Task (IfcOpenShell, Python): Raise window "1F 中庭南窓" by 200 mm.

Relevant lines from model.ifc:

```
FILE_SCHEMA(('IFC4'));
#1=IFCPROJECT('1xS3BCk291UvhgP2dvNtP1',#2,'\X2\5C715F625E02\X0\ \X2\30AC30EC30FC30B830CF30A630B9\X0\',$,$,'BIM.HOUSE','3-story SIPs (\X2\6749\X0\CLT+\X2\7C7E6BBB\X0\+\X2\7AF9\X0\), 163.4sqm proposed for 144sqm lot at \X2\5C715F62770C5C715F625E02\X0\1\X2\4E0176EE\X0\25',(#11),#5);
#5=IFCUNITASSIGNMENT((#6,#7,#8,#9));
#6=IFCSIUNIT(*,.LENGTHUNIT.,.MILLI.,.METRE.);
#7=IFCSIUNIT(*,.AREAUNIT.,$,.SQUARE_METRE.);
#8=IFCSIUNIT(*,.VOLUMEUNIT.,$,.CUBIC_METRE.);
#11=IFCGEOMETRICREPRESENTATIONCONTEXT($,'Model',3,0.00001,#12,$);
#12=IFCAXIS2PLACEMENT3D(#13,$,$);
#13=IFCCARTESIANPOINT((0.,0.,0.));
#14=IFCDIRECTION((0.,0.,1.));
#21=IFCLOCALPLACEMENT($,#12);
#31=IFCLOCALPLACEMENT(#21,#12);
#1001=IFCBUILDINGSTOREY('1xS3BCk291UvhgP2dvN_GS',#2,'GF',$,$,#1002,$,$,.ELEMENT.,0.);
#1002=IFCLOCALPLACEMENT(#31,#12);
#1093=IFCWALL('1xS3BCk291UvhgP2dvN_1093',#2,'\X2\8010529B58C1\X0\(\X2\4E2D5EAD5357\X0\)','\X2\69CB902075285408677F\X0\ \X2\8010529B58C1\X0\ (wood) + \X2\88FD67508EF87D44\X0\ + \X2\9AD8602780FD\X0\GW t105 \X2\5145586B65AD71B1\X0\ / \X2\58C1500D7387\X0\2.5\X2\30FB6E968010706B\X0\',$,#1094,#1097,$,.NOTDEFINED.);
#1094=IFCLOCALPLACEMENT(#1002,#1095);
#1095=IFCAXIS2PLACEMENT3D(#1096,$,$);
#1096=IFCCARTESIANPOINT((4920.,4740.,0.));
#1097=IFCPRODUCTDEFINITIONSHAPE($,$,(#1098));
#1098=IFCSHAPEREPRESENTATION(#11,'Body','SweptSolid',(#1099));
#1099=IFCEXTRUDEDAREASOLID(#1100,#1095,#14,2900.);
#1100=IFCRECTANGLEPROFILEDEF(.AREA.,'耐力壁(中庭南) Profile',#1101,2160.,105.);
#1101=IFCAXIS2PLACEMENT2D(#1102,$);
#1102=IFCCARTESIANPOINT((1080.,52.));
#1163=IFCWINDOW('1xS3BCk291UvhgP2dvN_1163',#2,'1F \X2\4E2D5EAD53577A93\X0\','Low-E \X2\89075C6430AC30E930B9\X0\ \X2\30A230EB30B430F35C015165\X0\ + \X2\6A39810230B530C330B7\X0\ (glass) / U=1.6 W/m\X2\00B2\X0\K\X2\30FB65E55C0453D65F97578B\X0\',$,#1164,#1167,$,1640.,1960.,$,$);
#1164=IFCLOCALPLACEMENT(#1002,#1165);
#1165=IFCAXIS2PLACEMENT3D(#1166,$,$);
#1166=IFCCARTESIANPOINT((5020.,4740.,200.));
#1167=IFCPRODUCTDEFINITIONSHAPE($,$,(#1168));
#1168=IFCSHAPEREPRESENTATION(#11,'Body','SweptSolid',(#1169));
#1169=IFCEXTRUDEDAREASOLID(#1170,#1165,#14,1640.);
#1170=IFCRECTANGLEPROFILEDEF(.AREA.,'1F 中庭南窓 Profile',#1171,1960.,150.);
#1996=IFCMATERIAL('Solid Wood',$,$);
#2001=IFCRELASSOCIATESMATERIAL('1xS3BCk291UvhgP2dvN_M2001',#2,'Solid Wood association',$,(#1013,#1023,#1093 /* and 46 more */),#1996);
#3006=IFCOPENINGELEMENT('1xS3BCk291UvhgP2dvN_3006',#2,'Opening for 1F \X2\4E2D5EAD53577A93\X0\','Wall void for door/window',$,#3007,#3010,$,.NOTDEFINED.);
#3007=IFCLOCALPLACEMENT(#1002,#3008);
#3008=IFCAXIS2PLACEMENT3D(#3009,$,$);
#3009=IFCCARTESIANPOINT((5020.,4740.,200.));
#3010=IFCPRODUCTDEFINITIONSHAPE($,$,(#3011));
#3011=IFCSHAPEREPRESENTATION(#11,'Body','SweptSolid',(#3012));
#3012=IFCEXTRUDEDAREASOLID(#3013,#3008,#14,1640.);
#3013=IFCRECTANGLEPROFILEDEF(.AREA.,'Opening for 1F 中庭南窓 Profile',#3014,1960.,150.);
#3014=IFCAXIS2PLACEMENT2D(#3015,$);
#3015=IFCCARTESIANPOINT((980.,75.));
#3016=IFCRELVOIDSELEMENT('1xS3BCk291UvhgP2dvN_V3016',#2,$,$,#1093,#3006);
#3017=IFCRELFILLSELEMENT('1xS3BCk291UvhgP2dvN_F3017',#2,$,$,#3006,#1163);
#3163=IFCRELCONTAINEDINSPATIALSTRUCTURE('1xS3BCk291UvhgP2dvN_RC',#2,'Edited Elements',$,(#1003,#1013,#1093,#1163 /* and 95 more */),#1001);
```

```python
import numpy as np
import ifcopenshell
import ifcopenshell.api.geometry
import ifcopenshell.util.placement
import ifcopenshell.util.unit

model = ifcopenshell.open("model.ifc")
unit_scale = ifcopenshell.util.unit.calculate_unit_scale(model)

window = model.by_guid("1xS3BCk291UvhgP2dvN_1163")
opening = window.FillsVoids[0].RelatingOpeningElement
dz = 200.0

shift = np.array([0.0, 0.0, dz])
# The window is not placed relative to its opening, so move both.
for product in (opening, window):
    matrix = ifcopenshell.util.placement.get_local_placement(product.ObjectPlacement)
    matrix[:3, 3] += shift
    ifcopenshell.api.geometry.edit_object_placement(model, product=product, matrix=matrix, is_si=False)

print(f"moved by {dz * unit_scale:+.3f} m")

model.write("model_updated.ifc")
```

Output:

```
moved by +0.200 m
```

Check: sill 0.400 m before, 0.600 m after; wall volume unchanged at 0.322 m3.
